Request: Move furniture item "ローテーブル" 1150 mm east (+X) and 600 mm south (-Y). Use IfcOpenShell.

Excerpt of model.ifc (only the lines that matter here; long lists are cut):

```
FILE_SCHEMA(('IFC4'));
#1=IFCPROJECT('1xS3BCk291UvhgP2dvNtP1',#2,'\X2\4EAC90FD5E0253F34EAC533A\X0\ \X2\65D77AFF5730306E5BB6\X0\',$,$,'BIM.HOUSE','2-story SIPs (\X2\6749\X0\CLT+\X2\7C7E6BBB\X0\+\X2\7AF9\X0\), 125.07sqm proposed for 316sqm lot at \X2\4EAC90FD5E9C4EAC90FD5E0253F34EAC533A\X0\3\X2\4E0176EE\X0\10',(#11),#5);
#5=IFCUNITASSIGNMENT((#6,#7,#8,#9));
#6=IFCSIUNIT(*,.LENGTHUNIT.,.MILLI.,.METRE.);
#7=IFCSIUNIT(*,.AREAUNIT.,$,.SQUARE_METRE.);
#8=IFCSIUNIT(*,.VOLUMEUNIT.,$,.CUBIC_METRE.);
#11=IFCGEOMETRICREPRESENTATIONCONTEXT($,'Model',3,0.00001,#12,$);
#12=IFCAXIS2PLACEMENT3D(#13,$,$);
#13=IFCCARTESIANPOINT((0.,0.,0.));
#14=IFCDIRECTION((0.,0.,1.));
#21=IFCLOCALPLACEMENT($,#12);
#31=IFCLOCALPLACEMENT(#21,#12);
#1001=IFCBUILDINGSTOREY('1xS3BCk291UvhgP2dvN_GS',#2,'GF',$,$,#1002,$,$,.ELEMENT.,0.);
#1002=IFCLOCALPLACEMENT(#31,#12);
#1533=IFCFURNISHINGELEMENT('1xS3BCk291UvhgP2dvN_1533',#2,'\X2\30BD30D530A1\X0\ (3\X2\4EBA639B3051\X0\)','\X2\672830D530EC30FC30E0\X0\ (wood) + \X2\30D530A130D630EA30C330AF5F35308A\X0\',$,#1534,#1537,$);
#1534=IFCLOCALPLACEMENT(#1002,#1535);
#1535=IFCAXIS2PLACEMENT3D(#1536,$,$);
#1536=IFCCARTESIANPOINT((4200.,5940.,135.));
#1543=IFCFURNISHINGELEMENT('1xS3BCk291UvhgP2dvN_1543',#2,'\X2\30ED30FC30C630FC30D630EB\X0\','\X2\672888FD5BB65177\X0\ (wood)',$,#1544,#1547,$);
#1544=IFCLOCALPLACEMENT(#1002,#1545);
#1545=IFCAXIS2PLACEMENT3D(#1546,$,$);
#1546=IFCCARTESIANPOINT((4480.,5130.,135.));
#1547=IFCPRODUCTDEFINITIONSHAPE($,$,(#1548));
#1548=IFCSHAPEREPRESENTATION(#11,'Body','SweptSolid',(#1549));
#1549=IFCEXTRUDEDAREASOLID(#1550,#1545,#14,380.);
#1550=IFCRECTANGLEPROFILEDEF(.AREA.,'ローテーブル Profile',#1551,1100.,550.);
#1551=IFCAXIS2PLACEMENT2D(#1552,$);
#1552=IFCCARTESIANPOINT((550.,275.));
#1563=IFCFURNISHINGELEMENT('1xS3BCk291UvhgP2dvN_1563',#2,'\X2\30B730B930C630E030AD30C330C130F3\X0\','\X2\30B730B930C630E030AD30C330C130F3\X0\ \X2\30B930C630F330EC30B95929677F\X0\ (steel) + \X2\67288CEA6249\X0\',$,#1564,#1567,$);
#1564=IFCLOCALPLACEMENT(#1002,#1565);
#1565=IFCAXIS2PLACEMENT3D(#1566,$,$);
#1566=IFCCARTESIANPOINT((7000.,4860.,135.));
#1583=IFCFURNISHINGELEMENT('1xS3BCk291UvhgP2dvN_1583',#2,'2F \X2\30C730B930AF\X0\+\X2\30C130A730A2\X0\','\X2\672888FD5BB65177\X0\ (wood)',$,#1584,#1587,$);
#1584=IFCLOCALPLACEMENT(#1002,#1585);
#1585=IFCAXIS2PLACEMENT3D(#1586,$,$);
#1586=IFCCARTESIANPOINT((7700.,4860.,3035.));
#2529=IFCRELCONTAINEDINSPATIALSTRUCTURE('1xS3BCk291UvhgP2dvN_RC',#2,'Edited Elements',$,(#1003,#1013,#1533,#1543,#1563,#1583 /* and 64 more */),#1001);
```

```python
import ifcopenshell
import ifcopenshell.api.geometry
import ifcopenshell.util.placement
import ifcopenshell.util.unit

model = ifcopenshell.open("model.ifc")
unit_scale = ifcopenshell.util.unit.calculate_unit_scale(model)

item = model.by_guid("1xS3BCk291UvhgP2dvN_1543")
matrix = ifcopenshell.util.placement.get_local_placement(item.ObjectPlacement)
matrix[0, 3] += 1.15 / unit_scale
matrix[1, 3] -= 0.6 / unit_scale
ifcopenshell.api.geometry.edit_object_placement(model, product=item, matrix=matrix, is_si=False)

print(ifcopenshell.util.placement.get_local_placement(item.ObjectPlacement).round(3) + 0.0)

model.write("model_edited.ifc")
```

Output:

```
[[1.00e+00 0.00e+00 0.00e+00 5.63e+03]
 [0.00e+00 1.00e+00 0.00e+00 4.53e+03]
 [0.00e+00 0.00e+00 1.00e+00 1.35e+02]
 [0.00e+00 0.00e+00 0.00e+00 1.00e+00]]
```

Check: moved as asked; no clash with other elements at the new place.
